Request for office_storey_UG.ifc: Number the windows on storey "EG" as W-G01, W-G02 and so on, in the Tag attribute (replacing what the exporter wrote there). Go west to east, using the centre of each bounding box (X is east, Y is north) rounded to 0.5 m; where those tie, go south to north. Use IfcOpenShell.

First a look at what the model holds.

```python
import ifcopenshell
import ifcopenshell.util.element
import ifcopenshell.util.placement

model = ifcopenshell.open("office_storey_UG.ifc")
print(model.schema)
storey = next(s for s in model.by_type("IfcBuildingStorey") if s.Name == "EG")
windows = [e for e in ifcopenshell.util.element.get_decomposition(storey) if e.is_a("IfcWindow")]
for e in sorted(windows, key=lambda e: e.id()):
    origin = ifcopenshell.util.placement.get_local_placement(e.ObjectPlacement)[:3, 3]
    print(e.id(), e.Tag, e.Name, origin.round(2) + 0.0, sep=" | ")
```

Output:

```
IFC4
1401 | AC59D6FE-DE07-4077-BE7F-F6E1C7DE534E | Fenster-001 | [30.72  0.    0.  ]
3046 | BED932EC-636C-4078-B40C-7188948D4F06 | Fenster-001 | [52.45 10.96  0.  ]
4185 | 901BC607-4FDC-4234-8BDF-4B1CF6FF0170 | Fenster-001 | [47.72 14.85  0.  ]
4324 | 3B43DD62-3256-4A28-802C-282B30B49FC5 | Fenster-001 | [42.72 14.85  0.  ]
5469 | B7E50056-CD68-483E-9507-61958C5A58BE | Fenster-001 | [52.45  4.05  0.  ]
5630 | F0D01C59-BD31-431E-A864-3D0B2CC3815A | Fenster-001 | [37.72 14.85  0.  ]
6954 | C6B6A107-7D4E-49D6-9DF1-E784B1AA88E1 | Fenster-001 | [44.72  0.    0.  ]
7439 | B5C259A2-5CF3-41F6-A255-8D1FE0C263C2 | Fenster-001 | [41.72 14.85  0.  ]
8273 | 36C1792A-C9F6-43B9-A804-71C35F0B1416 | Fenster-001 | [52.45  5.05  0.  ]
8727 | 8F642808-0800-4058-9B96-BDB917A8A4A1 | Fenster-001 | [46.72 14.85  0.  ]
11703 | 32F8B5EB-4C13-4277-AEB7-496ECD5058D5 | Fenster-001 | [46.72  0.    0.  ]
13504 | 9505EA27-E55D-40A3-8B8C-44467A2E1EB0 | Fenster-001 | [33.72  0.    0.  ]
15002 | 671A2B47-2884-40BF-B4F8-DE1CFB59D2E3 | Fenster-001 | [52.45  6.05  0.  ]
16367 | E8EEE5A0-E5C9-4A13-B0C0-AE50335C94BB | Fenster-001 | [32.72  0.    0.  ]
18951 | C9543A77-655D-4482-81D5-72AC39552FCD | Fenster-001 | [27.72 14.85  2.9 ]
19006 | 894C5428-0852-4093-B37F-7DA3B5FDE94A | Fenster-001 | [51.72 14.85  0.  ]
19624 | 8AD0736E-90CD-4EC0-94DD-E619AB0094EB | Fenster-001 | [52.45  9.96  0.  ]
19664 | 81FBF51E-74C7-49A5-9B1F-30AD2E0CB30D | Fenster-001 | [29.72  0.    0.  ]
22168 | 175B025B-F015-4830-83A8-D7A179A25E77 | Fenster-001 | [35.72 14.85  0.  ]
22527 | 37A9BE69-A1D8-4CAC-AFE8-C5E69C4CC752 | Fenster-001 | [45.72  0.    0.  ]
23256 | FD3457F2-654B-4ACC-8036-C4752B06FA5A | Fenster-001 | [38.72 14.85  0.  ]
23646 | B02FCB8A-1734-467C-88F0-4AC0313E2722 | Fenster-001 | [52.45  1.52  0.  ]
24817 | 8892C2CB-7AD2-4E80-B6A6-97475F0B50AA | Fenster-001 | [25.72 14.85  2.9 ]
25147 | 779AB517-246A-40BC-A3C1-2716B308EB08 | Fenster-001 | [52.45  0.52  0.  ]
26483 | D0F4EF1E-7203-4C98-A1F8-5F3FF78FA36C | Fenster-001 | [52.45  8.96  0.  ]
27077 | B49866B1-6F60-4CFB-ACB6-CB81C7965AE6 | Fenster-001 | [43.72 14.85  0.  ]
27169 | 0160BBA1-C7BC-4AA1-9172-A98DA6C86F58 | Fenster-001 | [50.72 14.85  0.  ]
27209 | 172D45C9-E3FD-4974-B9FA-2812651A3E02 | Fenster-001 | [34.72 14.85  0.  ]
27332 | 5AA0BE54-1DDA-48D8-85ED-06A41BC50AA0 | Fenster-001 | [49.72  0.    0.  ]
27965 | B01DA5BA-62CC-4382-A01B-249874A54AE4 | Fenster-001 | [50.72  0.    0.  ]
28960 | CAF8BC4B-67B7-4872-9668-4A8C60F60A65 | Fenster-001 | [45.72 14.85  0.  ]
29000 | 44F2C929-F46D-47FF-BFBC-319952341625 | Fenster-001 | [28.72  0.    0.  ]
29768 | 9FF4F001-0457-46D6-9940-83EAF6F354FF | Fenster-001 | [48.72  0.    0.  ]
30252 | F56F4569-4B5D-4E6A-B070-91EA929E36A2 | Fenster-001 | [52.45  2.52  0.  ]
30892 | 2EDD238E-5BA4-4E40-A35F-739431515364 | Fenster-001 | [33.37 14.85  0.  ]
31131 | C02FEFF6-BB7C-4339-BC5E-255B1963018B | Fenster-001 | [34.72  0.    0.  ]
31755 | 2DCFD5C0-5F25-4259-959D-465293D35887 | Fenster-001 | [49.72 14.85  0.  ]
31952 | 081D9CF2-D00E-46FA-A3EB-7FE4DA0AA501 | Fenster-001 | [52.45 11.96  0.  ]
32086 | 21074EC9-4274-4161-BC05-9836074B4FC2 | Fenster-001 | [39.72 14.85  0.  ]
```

```python
import ifcopenshell
import ifcopenshell.geom
import ifcopenshell.util.element
import ifcopenshell.util.shape

model = ifcopenshell.open("office_storey_UG.ifc")
settings = ifcopenshell.geom.settings()
settings.set("use-world-coords", True)


def centre(element):
    shape = ifcopenshell.geom.create_shape(settings, element)
    return ifcopenshell.util.shape.get_bbox_centroid(shape.geometry)


storey = next(s for s in model.by_type("IfcBuildingStorey") if s.Name == "EG")
windows = [e for e in ifcopenshell.util.element.get_decomposition(storey) if e.is_a("IfcWindow")]

# Insertion points can sit at a corner or the storey origin, so sort by the geometry (in metres).
centres = {e: centre(e) for e in windows}
windows.sort(key=lambda e: (round(centres[e][0] / 0.5), centres[e][1]))

for i, e in enumerate(windows, start=1):
    number = f"W-G{i:02d}"
    e.Tag = number
    print(e.id(), number)

model.write("office_storey_UG_v2.ifc")
```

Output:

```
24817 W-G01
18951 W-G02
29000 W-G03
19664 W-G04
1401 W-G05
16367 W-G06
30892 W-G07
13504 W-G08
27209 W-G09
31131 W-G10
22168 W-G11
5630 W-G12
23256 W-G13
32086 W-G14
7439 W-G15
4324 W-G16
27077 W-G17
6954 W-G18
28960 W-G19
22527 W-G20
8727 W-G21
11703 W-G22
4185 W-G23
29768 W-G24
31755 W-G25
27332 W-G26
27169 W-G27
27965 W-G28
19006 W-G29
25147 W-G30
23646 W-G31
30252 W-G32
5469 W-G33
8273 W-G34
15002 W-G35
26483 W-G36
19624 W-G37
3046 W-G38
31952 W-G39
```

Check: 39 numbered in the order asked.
